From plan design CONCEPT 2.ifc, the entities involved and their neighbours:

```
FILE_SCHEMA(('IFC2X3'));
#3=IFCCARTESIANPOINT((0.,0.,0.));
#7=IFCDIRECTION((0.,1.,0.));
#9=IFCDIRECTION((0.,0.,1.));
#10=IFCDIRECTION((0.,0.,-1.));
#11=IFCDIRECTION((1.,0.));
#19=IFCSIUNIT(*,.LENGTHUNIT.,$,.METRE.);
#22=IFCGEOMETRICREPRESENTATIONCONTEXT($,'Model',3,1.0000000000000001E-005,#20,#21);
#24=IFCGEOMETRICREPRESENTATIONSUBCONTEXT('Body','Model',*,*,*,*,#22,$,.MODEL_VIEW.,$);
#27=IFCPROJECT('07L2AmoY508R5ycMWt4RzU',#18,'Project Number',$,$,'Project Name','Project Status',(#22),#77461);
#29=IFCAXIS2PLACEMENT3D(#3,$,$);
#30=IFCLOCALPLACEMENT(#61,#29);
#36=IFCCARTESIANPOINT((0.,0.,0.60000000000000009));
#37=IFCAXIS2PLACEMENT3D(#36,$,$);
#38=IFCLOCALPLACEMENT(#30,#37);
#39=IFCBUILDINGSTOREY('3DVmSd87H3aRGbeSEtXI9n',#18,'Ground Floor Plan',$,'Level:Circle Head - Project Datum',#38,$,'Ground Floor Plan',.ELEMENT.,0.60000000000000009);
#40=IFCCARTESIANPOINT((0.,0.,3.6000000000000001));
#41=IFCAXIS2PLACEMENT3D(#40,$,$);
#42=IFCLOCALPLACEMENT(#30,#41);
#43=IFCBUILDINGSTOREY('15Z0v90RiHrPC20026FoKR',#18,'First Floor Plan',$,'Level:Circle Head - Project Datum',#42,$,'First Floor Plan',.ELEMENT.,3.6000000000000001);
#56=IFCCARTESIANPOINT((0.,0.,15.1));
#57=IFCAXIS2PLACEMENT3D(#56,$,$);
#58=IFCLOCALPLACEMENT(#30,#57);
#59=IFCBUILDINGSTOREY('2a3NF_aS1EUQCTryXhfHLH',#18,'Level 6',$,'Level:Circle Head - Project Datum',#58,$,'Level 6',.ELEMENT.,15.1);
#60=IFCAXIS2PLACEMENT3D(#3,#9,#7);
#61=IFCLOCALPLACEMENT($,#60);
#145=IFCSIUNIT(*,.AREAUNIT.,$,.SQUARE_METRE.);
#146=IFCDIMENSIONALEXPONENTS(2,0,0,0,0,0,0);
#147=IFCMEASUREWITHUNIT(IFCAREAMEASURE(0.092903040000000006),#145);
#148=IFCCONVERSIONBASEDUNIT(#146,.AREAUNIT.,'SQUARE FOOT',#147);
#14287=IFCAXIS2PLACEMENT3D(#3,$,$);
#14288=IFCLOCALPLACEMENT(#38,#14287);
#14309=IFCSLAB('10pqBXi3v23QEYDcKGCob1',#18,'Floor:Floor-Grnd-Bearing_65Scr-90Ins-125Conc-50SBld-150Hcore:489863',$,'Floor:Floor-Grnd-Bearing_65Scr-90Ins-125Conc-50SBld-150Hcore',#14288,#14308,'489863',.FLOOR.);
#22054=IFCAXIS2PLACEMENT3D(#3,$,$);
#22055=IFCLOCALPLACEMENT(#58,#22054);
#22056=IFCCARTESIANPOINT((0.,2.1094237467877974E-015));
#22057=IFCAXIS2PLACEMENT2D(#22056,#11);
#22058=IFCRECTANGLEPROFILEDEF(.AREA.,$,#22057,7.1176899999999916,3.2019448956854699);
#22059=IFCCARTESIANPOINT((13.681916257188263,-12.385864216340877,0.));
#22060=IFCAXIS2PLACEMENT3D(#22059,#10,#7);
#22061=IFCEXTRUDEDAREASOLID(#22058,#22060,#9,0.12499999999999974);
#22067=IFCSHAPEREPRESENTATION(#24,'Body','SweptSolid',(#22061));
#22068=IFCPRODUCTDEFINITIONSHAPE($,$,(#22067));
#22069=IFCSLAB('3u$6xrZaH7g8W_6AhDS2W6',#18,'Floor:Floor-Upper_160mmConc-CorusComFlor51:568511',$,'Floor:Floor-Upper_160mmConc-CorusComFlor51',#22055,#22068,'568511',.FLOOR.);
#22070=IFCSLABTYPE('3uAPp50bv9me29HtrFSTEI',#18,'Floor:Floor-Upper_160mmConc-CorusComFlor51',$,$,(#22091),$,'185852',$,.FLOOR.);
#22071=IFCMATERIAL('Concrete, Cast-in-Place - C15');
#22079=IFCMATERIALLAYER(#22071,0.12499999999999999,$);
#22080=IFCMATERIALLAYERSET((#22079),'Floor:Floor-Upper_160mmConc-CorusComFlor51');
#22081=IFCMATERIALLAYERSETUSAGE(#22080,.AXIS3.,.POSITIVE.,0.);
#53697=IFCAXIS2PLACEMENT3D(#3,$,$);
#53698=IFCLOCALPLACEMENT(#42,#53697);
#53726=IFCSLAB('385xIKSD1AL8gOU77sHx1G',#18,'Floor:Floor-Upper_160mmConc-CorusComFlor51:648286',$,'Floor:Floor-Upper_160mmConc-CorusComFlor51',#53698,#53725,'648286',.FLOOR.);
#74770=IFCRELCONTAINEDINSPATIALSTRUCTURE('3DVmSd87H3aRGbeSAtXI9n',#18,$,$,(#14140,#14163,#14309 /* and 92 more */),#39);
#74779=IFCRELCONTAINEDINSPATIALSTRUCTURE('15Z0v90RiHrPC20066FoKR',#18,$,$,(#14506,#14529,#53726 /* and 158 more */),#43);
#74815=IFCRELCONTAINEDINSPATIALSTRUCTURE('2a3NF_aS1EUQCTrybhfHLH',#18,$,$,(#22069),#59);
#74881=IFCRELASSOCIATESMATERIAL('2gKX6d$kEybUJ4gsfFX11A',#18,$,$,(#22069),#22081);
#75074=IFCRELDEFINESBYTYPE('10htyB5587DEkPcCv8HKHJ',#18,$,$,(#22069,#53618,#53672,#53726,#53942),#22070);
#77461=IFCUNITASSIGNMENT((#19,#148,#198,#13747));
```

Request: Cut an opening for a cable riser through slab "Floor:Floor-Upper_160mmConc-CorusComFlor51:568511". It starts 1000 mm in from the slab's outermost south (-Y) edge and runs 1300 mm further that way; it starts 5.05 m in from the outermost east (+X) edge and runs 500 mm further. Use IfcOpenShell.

```python
import numpy as np
import ifcopenshell
import ifcopenshell.api.feature
import ifcopenshell.api.geometry
import ifcopenshell.api.root
import ifcopenshell.geom
import ifcopenshell.util.placement
import ifcopenshell.util.representation
import ifcopenshell.util.shape
import ifcopenshell.util.unit

model = ifcopenshell.open("plan design CONCEPT 2.ifc")
unit_scale = ifcopenshell.util.unit.calculate_unit_scale(model)
settings = ifcopenshell.geom.settings()


def volume(element):
    """Net volume in cubic metres, openings subtracted."""
    shape = ifcopenshell.geom.create_shape(settings, element)
    return ifcopenshell.util.shape.get_volume(shape.geometry)


slab = model.by_guid("3u$6xrZaH7g8W_6AhDS2W6")
before = volume(slab)

# Extent in the slab's own axes, in metres. The edges named are its -X and -Y sides.
slab_shape = ifcopenshell.geom.create_shape(settings, slab)
vertices = ifcopenshell.util.shape.get_vertices(slab_shape.geometry)
x_min, y_min, bottom = vertices.min(axis=0)
top = vertices[:, 2].max()

opening = ifcopenshell.api.root.create_entity(model, ifc_class="IfcOpeningElement", name="Cable riser opening")
context = ifcopenshell.util.representation.get_context(model, "Model", "Body", "MODEL_VIEW")
width, depth = 1.3, 0.5
outline = [(0.0, 0.0), (width, 0.0), (width, depth), (0.0, depth), (0.0, 0.0)]
# Overshoot both faces by 50 mm so the cut is clean.
shape = ifcopenshell.api.geometry.add_slab_representation(
    model, context=context, depth=top - bottom + 0.1, polyline=outline
)
ifcopenshell.api.geometry.assign_representation(model, product=opening, representation=shape)

matrix = ifcopenshell.util.placement.get_local_placement(slab.ObjectPlacement)
matrix[:, 3] = matrix @ np.append(np.array([x_min + 1, y_min + 5.05, bottom - 0.05]) / unit_scale, 1.0)
ifcopenshell.api.geometry.edit_object_placement(model, product=opening, matrix=matrix, is_si=False)
ifcopenshell.api.feature.add_feature(model, feature=opening, element=slab)

after = volume(slab)

print(f"slab volume {before:.3f} -> {after:.3f} m3")

model.write("plan design CONCEPT 2-out.ifc")
```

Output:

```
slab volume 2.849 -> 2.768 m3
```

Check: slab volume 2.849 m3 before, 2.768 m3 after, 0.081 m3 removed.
